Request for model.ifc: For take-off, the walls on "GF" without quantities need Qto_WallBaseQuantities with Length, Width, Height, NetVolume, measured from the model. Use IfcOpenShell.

First a look at what the model holds.

```python
import ifcopenshell
import ifcopenshell.util.element
import ifcopenshell.util.unit

model = ifcopenshell.open("model.ifc")
print(model.schema)
for unit_type in ("LENGTHUNIT", "AREAUNIT", "VOLUMEUNIT"):
    print(unit_type, ifcopenshell.util.unit.calculate_unit_scale(model, unit_type))
storey = next(s for s in model.by_type("IfcBuildingStorey") if s.Name == "GF")
walls = [e for e in ifcopenshell.util.element.get_decomposition(storey) if e.is_a("IfcWall")]
for e in sorted(walls, key=lambda e: e.id()):
    print(e.id(), e.is_a(), e.Name, list(ifcopenshell.util.element.get_psets(e, qtos_only=True)), sep=" | ")
```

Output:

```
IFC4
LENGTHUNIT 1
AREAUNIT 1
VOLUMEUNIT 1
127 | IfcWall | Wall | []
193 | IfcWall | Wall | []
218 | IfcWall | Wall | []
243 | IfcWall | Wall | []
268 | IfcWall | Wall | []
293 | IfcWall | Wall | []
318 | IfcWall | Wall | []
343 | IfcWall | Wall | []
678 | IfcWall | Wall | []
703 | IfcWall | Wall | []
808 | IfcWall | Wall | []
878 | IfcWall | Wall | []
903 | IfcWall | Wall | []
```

```python
import ifcopenshell
import ifcopenshell.api.pset
import ifcopenshell.geom
import ifcopenshell.util.element
import ifcopenshell.util.shape
import ifcopenshell.util.unit

model = ifcopenshell.open("model.ifc")
unit_scale = ifcopenshell.util.unit.calculate_unit_scale(model)
volume_scale = ifcopenshell.util.unit.calculate_unit_scale(model, "VOLUMEUNIT")
settings = ifcopenshell.geom.settings()

storey = next(s for s in model.by_type("IfcBuildingStorey") if s.Name == "GF")
walls = [e for e in ifcopenshell.util.element.get_decomposition(storey) if e.is_a("IfcWall")]

for e in sorted(walls, key=lambda e: e.id()):
    if ifcopenshell.util.element.get_psets(e, qtos_only=True, should_inherit=False):
        continue
    # Geometry comes back in metres, in the element's own axes.
    shape = ifcopenshell.geom.create_shape(settings, e)
    values = {
        "Length": ifcopenshell.util.shape.get_x(shape.geometry) / unit_scale,
        "Width": ifcopenshell.util.shape.get_y(shape.geometry) / unit_scale,
        "Height": ifcopenshell.util.shape.get_z(shape.geometry) / unit_scale,
        "NetVolume": ifcopenshell.util.shape.get_volume(shape.geometry) / volume_scale,
    }
    qto = ifcopenshell.api.pset.add_qto(model, product=e, name="Qto_WallBaseQuantities")
    ifcopenshell.api.pset.edit_qto(model, qto=qto, properties=values)
    print(e.id(), {k: round(v, 3) for k, v in values.items()})

model.write("model_edited.ifc")
```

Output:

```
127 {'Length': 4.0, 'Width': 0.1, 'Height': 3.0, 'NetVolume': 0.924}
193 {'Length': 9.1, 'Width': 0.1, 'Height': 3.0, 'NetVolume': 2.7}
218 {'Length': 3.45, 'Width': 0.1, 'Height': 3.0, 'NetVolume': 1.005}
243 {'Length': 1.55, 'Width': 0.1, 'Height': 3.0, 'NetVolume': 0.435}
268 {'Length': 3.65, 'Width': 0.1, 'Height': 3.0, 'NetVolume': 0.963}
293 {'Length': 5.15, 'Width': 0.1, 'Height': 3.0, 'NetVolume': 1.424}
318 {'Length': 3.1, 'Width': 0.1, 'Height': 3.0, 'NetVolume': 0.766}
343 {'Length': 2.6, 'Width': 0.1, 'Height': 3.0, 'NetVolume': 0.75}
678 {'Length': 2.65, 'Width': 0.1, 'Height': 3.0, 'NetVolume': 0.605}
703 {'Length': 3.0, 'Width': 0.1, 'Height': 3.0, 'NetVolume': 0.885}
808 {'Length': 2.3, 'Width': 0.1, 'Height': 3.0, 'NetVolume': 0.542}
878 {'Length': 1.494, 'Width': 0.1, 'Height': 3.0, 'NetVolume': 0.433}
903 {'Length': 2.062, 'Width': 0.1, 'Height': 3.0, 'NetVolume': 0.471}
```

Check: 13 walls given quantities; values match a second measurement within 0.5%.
